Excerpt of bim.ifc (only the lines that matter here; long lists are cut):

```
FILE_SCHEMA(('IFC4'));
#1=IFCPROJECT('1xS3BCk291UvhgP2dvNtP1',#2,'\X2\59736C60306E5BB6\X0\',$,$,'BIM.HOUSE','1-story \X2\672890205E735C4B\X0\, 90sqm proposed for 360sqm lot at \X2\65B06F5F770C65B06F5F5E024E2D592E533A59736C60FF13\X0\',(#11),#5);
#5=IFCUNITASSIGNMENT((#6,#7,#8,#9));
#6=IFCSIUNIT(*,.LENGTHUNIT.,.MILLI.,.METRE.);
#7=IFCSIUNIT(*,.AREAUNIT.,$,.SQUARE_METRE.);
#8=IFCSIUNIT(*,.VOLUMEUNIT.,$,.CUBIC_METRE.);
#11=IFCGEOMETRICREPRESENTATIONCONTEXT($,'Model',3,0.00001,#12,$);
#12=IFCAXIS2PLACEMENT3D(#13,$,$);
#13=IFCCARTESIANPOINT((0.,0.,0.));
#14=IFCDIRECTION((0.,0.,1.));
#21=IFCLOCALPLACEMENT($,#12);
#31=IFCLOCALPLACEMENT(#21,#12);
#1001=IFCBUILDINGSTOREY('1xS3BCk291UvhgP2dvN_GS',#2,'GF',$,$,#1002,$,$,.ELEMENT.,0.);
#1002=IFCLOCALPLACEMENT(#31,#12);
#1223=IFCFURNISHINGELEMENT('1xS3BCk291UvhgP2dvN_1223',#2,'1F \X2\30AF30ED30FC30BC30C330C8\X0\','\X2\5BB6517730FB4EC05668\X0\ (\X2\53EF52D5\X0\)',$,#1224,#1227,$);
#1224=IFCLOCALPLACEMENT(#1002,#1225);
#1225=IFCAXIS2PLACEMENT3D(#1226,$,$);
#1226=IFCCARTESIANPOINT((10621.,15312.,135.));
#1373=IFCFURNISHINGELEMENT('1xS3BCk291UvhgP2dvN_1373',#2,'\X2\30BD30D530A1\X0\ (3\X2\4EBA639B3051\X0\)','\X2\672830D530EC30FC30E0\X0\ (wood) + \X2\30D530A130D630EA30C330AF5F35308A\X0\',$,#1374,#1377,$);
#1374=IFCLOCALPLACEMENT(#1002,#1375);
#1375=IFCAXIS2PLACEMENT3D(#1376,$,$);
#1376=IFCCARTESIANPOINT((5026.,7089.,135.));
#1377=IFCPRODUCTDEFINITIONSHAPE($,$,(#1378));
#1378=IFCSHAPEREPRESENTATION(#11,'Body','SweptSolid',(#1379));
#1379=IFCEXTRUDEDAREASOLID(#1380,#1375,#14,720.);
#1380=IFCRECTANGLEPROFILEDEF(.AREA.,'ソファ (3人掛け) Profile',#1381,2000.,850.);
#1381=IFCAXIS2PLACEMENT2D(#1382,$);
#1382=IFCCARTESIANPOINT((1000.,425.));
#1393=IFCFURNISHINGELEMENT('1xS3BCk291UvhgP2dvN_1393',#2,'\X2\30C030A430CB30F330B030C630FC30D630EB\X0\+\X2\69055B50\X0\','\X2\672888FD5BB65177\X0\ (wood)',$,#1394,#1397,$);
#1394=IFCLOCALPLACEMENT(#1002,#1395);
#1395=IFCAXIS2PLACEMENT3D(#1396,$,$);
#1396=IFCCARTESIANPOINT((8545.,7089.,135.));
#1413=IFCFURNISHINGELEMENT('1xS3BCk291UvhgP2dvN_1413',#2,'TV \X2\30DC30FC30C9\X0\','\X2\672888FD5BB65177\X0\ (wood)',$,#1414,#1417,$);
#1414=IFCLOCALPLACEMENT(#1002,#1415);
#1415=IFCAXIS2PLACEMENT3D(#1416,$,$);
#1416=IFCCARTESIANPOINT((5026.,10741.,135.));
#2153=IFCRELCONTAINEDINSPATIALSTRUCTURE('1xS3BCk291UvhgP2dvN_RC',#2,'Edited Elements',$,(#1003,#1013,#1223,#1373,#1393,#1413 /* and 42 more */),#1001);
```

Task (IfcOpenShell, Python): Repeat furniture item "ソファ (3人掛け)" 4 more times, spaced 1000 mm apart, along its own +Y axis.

```python
import ifcopenshell
import ifcopenshell.api.geometry
import ifcopenshell.api.root
import ifcopenshell.util.element
import ifcopenshell.util.placement

model = ifcopenshell.open("bim.ifc")


def reuse_history(source, copy):
    """copy_class also copies each property set's owner history, people and application; keep the originals."""
    for rel in copy.IsDefinedBy:
        if rel.is_a("IfcRelDefinesByProperties") and (history := rel.RelatingPropertyDefinition.OwnerHistory):
            rel.RelatingPropertyDefinition.OwnerHistory = source.OwnerHistory
            ifcopenshell.util.element.remove_deep2(model, history)


source = model.by_guid("1xS3BCk291UvhgP2dvN_1373")
base = ifcopenshell.util.placement.get_local_placement(source.ObjectPlacement)
step = base[:3, 1] * 1000.0

for i in range(1, 5):
    copy = ifcopenshell.api.root.copy_class(model, product=source)
    copy.Representation = ifcopenshell.util.element.copy_deep(
        model, source.Representation, exclude=["IfcGeometricRepresentationContext", "IfcRepresentationMap"]
    )
    reuse_history(source, copy)
    matrix = base.copy()
    matrix[:3, 3] += i * step
    print("added at", matrix[:3, 3].round(3) + 0.0)
    ifcopenshell.api.geometry.edit_object_placement(model, product=copy, matrix=matrix, is_si=False)

model.write("bim_rev.ifc")
```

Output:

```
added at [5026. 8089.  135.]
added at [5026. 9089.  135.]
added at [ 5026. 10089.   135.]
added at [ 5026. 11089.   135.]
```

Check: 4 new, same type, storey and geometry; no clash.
